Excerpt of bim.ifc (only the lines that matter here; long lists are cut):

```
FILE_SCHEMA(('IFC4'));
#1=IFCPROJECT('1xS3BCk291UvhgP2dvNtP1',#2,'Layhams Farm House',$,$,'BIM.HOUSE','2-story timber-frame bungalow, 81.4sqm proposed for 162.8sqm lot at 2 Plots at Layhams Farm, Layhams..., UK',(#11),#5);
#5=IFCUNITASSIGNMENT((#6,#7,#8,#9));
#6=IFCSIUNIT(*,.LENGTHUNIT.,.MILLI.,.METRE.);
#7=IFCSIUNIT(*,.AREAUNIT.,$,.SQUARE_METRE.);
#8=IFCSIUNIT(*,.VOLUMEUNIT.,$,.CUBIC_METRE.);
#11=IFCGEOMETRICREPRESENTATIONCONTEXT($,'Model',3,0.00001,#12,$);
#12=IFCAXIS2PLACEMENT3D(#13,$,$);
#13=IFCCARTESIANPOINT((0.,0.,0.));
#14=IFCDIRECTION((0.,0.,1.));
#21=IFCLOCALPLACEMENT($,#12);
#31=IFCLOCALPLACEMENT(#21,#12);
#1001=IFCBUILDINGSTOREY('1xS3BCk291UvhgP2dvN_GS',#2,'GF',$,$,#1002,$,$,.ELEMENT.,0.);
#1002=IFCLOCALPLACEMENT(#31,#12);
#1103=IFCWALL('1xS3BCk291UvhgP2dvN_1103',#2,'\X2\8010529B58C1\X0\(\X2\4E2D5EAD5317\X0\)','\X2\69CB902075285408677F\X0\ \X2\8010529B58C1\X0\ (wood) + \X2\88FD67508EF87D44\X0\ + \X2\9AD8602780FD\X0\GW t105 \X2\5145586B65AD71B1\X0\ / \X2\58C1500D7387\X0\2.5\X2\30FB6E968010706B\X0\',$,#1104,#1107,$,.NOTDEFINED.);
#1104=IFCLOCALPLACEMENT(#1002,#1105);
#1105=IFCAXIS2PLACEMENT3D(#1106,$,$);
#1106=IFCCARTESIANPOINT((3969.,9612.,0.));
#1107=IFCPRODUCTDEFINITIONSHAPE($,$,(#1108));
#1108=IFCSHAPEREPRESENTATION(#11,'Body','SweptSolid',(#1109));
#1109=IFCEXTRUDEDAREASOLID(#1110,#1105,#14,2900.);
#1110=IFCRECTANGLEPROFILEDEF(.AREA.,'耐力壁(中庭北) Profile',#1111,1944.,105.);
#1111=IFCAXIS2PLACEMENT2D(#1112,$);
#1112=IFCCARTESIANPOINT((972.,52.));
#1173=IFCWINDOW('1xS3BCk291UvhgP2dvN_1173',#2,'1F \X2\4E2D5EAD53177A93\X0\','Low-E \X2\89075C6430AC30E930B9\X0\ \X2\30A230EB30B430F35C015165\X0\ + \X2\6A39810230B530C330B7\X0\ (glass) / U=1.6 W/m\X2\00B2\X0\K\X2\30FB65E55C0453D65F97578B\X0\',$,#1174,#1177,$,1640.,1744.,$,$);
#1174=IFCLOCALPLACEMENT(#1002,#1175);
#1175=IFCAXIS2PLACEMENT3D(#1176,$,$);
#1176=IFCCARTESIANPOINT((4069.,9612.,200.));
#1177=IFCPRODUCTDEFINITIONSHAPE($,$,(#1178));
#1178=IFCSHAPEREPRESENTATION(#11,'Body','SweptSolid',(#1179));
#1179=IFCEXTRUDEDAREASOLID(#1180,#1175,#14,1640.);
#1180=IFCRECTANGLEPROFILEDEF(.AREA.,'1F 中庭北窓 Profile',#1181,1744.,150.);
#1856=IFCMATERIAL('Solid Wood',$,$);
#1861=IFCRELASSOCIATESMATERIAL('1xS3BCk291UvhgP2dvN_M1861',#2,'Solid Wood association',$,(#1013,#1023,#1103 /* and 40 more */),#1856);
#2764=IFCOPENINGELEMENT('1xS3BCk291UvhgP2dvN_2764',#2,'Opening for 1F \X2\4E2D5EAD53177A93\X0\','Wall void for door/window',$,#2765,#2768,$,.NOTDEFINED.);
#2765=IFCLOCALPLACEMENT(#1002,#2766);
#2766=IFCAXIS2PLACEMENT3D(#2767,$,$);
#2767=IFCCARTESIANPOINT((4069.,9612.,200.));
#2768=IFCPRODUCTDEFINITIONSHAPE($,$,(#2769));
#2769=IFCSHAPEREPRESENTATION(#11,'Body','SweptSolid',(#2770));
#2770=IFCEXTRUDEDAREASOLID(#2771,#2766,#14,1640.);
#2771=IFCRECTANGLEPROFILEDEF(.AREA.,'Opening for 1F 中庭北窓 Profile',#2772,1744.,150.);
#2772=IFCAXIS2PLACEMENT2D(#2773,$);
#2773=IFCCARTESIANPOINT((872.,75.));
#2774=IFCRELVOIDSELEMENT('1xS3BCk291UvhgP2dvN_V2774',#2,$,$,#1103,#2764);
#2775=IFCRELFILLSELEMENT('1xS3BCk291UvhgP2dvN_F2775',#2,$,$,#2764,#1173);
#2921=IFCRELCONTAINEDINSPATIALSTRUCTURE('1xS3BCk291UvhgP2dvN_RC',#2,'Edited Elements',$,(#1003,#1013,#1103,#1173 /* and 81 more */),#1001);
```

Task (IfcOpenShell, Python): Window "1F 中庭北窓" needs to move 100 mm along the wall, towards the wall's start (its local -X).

```python
import ifcopenshell
import ifcopenshell.api.geometry
import ifcopenshell.util.placement

model = ifcopenshell.open("bim.ifc")

window = model.by_guid("1xS3BCk291UvhgP2dvN_1173")
opening = window.FillsVoids[0].RelatingOpeningElement
wall = opening.VoidsElements[0].RelatingBuildingElement

wall_matrix = ifcopenshell.util.placement.get_local_placement(wall.ObjectPlacement)
shift = wall_matrix[:3, 0] * -100.0
before = ifcopenshell.util.placement.get_local_placement(window.ObjectPlacement)[:3, 3].copy()

# The window is not placed relative to its opening, so move both.
for product in (opening, window):
    matrix = ifcopenshell.util.placement.get_local_placement(product.ObjectPlacement)
    matrix[:3, 3] += shift
    ifcopenshell.api.geometry.edit_object_placement(model, product=product, matrix=matrix, is_si=False)

after = ifcopenshell.util.placement.get_local_placement(window.ObjectPlacement)[:3, 3]
print("window moved by", (after - before).round(3) + 0.0)

model.write("bim_rev.ifc")
```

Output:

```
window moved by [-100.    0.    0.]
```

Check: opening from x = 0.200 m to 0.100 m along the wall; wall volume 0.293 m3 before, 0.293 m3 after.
